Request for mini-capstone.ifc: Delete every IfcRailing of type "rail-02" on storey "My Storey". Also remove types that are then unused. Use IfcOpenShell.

First a look at what the model holds.

```python
import ifcopenshell
import ifcopenshell.util.element

model = ifcopenshell.open("mini-capstone.ifc")
print(model.schema)
storey = next(s for s in model.by_type("IfcBuildingStorey") if s.Name == "My Storey")
railings = [e for e in ifcopenshell.util.element.get_decomposition(storey) if e.is_a("IfcRailing")]
seen = {}
for e in railings:
    element_type = ifcopenshell.util.element.get_type(e)
    name = element_type.Name if element_type not in (None, e) else None
    seen[name] = seen.get(name, 0) + 1
for name, count in sorted(seen.items(), key=str):
    print(count, "x", name)
```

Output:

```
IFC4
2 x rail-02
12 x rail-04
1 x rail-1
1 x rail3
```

```python
import ifcopenshell
import ifcopenshell.api.root
import ifcopenshell.util.element

model = ifcopenshell.open("mini-capstone.ifc")

storey = next(s for s in model.by_type("IfcBuildingStorey") if s.Name == "My Storey")
railings = [e for e in ifcopenshell.util.element.get_decomposition(storey) if e.is_a("IfcRailing")]
targets = [e for e in railings if (t := ifcopenshell.util.element.get_type(e)) not in (None, e) and t.Name == "rail-02"]
types = {ifcopenshell.util.element.get_type(e) for e in targets} - {None, *targets}

for e in targets:
    ifcopenshell.api.root.remove_product(model, product=e)
print(len(targets), "removed")

unused = [t for t in types if not ifcopenshell.util.element.get_types(t)]
for t in unused:
    ifcopenshell.api.root.remove_product(model, product=t)
print(len(unused), "unused types removed")

model.write("mini-capstone_updated.ifc")
```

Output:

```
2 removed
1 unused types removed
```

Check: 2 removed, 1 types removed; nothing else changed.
